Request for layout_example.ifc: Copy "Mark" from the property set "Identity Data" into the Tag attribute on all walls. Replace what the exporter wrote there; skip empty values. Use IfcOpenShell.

First a look at what the model holds.

```python
import ifcopenshell
import ifcopenshell.util.element

model = ifcopenshell.open("layout_example.ifc")
print(model.schema)
walls = model.by_type("IfcWall")
print(len(walls), "walls")
for e in walls[:8]:
    source = ifcopenshell.util.element.get_pset(e, "Identity Data", "Mark")
    target = e.Tag
    print(e.id(), repr(source), repr(target), sep=" | ")
```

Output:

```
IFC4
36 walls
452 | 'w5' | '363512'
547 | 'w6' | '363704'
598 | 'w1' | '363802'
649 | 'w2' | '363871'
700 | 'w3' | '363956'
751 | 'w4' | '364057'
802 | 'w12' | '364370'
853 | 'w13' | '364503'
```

```python
import ifcopenshell
import ifcopenshell.util.element

model = ifcopenshell.open("layout_example.ifc")

count = 0
for e in model.by_type("IfcWall"):
    value = ifcopenshell.util.element.get_pset(e, "Identity Data", "Mark")
    current = e.Tag
    if not value or not value.strip() or current == value:
        continue
    e.Tag = value
    count += 1

print(count, "walls updated")

model.write("layout_example_rev.ifc")
```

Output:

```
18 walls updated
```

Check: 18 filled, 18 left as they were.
